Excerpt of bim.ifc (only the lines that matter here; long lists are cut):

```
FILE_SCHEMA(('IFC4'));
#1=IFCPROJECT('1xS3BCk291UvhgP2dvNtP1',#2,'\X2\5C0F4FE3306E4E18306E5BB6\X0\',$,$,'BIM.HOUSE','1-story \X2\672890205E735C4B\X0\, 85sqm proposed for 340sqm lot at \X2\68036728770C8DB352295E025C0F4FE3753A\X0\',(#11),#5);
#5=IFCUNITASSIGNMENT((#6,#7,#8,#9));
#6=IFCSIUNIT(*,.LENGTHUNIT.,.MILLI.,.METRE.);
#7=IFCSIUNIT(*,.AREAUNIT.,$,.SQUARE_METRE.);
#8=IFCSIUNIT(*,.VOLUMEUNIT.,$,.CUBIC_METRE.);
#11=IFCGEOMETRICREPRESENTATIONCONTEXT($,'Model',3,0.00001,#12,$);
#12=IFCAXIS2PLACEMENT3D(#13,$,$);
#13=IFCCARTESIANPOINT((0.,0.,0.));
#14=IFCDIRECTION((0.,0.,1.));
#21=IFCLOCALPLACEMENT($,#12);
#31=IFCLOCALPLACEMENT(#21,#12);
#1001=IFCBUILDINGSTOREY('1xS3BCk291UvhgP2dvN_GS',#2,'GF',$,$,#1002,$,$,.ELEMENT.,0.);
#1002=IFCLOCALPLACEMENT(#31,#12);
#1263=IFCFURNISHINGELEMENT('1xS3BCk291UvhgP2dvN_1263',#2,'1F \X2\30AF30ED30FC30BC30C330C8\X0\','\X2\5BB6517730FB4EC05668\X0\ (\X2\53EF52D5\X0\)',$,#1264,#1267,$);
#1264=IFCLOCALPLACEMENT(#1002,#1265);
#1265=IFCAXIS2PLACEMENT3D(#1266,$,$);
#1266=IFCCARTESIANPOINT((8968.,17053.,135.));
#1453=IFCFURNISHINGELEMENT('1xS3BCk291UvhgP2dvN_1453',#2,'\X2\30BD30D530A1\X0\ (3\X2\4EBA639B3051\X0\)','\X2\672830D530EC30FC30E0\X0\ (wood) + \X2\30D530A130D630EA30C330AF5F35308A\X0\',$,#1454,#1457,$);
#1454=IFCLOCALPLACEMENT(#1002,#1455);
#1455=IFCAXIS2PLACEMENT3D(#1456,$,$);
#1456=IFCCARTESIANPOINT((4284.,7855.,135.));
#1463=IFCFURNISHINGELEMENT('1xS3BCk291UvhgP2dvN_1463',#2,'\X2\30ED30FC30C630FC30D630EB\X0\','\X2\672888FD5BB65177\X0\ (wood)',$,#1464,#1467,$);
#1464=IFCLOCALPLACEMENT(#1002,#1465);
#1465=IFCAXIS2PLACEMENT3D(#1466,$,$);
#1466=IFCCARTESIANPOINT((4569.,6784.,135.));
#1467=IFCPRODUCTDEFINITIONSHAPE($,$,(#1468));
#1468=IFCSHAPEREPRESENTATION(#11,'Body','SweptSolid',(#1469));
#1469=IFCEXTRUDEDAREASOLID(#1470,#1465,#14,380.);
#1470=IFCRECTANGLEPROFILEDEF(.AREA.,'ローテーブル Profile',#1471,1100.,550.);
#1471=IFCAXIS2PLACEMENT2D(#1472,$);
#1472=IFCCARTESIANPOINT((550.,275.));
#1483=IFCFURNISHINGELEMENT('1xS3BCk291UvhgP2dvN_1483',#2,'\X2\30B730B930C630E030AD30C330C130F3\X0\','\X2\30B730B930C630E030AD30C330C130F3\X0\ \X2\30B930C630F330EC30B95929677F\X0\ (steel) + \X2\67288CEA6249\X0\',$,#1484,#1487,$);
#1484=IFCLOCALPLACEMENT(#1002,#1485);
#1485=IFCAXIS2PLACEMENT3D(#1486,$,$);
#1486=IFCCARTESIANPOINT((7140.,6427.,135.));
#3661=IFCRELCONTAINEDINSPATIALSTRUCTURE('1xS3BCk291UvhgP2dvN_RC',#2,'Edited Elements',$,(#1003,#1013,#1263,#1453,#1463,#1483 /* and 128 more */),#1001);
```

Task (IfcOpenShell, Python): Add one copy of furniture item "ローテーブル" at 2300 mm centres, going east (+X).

```python
import numpy as np
import ifcopenshell
import ifcopenshell.api.geometry
import ifcopenshell.api.root
import ifcopenshell.util.element
import ifcopenshell.util.placement
import ifcopenshell.util.unit

model = ifcopenshell.open("bim.ifc")
unit_scale = ifcopenshell.util.unit.calculate_unit_scale(model)


def reuse_history(source, copy):
    """copy_class also copies each property set's owner history, people and application; keep the originals."""
    for rel in copy.IsDefinedBy:
        if rel.is_a("IfcRelDefinesByProperties") and (history := rel.RelatingPropertyDefinition.OwnerHistory):
            rel.RelatingPropertyDefinition.OwnerHistory = source.OwnerHistory
            ifcopenshell.util.element.remove_deep2(model, history)


source = model.by_id(1463)
base = ifcopenshell.util.placement.get_local_placement(source.ObjectPlacement)
step = np.array([1.0, 0.0, 0.0]) * 2.3 / unit_scale

for i in range(1, 2):
    copy = ifcopenshell.api.root.copy_class(model, product=source)
    copy.Representation = ifcopenshell.util.element.copy_deep(
        model, source.Representation, exclude=["IfcGeometricRepresentationContext", "IfcRepresentationMap"]
    )
    reuse_history(source, copy)
    matrix = base.copy()
    matrix[:3, 3] += i * step
    print("added at", matrix[:3, 3].round(3) + 0.0)
    ifcopenshell.api.geometry.edit_object_placement(model, product=copy, matrix=matrix, is_si=False)

model.write("bim-out.ifc")
```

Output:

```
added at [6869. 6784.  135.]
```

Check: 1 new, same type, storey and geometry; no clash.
